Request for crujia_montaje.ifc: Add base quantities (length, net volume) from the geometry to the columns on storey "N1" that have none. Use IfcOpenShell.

First a look at what the model holds.

```python
import ifcopenshell
import ifcopenshell.util.element
import ifcopenshell.util.unit

model = ifcopenshell.open("crujia_montaje.ifc")
print(model.schema)
for unit_type in ("LENGTHUNIT", "AREAUNIT", "VOLUMEUNIT"):
    print(unit_type, ifcopenshell.util.unit.calculate_unit_scale(model, unit_type))
storey = next(s for s in model.by_type("IfcBuildingStorey") if s.Name == "N1")
columns = [e for e in ifcopenshell.util.element.get_decomposition(storey) if e.is_a("IfcColumn")]
for e in sorted(columns, key=lambda e: e.id()):
    print(e.id(), e.is_a(), e.Name, list(ifcopenshell.util.element.get_psets(e, qtos_only=True)), sep=" | ")
```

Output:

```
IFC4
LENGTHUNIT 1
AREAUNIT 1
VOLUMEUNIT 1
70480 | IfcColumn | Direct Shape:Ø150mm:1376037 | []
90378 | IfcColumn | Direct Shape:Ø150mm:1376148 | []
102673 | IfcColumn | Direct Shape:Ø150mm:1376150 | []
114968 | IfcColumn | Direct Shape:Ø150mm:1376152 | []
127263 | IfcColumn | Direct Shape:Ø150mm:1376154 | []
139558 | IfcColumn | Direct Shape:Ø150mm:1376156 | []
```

```python
import ifcopenshell
import ifcopenshell.api.pset
import ifcopenshell.geom
import ifcopenshell.util.element
import ifcopenshell.util.shape
import ifcopenshell.util.unit

model = ifcopenshell.open("crujia_montaje.ifc")
unit_scale = ifcopenshell.util.unit.calculate_unit_scale(model)
volume_scale = ifcopenshell.util.unit.calculate_unit_scale(model, "VOLUMEUNIT")
settings = ifcopenshell.geom.settings()

storey = next(s for s in model.by_type("IfcBuildingStorey") if s.Name == "N1")
columns = [e for e in ifcopenshell.util.element.get_decomposition(storey) if e.is_a("IfcColumn")]

for e in sorted(columns, key=lambda e: e.id()):
    if ifcopenshell.util.element.get_psets(e, qtos_only=True, should_inherit=False):
        continue
    # Geometry comes back in metres, in the element's own axes.
    shape = ifcopenshell.geom.create_shape(settings, e)
    values = {
        "Length": ifcopenshell.util.shape.get_z(shape.geometry) / unit_scale,
        "NetVolume": ifcopenshell.util.shape.get_volume(shape.geometry) / volume_scale,
    }
    qto = ifcopenshell.api.pset.add_qto(model, product=e, name="Qto_ColumnBaseQuantities")
    ifcopenshell.api.pset.edit_qto(model, qto=qto, properties=values)
    print(e.id(), {k: round(v, 3) for k, v in values.items()})

model.write("crujia_montaje-out.ifc")
```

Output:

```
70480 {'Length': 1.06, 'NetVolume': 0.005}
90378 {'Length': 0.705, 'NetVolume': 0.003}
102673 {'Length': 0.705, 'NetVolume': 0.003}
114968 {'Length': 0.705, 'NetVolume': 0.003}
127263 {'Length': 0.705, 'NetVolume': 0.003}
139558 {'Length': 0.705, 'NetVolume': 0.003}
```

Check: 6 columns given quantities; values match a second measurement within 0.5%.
